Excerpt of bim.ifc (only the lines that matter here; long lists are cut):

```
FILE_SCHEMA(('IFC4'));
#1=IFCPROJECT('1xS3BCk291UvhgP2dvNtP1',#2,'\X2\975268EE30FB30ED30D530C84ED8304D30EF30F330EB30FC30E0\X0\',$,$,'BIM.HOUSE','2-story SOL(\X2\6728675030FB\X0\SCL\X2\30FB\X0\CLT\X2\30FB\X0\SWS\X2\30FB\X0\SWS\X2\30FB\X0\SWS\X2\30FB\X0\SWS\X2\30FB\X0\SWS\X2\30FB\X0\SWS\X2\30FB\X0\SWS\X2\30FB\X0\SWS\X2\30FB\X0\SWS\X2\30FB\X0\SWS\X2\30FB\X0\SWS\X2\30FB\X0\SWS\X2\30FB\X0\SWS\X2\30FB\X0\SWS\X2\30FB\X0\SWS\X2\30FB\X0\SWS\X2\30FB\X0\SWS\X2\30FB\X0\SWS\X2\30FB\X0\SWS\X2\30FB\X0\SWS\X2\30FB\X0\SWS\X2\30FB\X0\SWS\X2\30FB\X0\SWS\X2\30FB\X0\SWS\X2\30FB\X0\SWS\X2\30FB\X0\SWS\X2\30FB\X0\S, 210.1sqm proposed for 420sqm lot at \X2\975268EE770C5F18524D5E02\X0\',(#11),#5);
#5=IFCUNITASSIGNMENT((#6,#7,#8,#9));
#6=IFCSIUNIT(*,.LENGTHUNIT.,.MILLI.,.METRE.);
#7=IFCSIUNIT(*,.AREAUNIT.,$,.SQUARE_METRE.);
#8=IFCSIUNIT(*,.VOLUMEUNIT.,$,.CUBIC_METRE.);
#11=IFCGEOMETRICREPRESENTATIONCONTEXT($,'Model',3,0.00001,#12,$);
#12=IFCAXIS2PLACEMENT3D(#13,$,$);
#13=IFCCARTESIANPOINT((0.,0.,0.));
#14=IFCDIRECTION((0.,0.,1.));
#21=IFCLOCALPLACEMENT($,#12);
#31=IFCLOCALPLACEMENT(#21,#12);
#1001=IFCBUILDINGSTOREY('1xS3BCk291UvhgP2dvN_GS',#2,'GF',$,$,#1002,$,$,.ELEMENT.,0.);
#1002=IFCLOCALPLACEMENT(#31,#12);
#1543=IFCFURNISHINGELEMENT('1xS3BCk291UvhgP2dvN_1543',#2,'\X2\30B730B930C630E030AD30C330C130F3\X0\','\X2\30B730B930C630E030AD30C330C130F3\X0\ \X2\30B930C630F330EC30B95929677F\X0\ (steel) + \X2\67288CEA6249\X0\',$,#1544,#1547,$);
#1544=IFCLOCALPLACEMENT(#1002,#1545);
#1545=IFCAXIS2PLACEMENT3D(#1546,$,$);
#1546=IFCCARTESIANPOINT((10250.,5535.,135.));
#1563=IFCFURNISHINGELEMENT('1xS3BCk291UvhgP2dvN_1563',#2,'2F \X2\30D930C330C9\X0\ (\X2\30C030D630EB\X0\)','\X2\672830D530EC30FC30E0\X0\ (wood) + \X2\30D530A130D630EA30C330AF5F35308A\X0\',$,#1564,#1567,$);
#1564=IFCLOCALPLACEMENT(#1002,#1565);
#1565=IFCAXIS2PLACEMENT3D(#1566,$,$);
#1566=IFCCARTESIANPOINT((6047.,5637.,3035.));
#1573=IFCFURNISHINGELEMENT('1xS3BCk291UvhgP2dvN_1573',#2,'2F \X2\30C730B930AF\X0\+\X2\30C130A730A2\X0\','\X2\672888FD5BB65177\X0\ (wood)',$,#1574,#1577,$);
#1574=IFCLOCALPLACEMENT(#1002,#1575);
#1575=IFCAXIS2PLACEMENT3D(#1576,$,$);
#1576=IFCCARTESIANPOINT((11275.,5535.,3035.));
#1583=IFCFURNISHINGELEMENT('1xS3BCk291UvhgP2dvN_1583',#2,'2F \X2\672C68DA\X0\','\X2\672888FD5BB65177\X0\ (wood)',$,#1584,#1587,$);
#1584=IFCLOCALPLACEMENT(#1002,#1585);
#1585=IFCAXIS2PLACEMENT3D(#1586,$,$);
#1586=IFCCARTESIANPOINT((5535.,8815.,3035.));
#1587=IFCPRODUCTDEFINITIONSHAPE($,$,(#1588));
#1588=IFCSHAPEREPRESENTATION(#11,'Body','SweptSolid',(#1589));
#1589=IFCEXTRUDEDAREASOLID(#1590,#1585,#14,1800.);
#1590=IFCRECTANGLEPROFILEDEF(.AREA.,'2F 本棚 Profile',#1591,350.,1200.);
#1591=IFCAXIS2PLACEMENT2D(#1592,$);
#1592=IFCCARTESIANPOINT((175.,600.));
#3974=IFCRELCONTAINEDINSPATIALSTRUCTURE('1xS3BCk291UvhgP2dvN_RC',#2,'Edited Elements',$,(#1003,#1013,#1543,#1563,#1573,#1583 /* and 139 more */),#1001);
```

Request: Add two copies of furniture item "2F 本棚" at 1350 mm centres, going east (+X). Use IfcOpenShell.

```python
import numpy as np
import ifcopenshell
import ifcopenshell.api.geometry
import ifcopenshell.api.root
import ifcopenshell.util.element
import ifcopenshell.util.placement
import ifcopenshell.util.unit

model = ifcopenshell.open("bim.ifc")
unit_scale = ifcopenshell.util.unit.calculate_unit_scale(model)


def reuse_history(source, copy):
    """copy_class also copies each property set's owner history, people and application; keep the originals."""
    for rel in copy.IsDefinedBy:
        if rel.is_a("IfcRelDefinesByProperties") and (history := rel.RelatingPropertyDefinition.OwnerHistory):
            rel.RelatingPropertyDefinition.OwnerHistory = source.OwnerHistory
            ifcopenshell.util.element.remove_deep2(model, history)


source = model.by_guid("1xS3BCk291UvhgP2dvN_1583")
base = ifcopenshell.util.placement.get_local_placement(source.ObjectPlacement)
step = np.array([1.0, 0.0, 0.0]) * 1.35 / unit_scale

for i in range(1, 3):
    copy = ifcopenshell.api.root.copy_class(model, product=source)
    copy.Representation = ifcopenshell.util.element.copy_deep(
        model, source.Representation, exclude=["IfcGeometricRepresentationContext", "IfcRepresentationMap"]
    )
    reuse_history(source, copy)
    matrix = base.copy()
    matrix[:3, 3] += i * step
    print("added at", matrix[:3, 3].round(3) + 0.0)
    ifcopenshell.api.geometry.edit_object_placement(model, product=copy, matrix=matrix, is_si=False)

model.write("bim-out.ifc")
```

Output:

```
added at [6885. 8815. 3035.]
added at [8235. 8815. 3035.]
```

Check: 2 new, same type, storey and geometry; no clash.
